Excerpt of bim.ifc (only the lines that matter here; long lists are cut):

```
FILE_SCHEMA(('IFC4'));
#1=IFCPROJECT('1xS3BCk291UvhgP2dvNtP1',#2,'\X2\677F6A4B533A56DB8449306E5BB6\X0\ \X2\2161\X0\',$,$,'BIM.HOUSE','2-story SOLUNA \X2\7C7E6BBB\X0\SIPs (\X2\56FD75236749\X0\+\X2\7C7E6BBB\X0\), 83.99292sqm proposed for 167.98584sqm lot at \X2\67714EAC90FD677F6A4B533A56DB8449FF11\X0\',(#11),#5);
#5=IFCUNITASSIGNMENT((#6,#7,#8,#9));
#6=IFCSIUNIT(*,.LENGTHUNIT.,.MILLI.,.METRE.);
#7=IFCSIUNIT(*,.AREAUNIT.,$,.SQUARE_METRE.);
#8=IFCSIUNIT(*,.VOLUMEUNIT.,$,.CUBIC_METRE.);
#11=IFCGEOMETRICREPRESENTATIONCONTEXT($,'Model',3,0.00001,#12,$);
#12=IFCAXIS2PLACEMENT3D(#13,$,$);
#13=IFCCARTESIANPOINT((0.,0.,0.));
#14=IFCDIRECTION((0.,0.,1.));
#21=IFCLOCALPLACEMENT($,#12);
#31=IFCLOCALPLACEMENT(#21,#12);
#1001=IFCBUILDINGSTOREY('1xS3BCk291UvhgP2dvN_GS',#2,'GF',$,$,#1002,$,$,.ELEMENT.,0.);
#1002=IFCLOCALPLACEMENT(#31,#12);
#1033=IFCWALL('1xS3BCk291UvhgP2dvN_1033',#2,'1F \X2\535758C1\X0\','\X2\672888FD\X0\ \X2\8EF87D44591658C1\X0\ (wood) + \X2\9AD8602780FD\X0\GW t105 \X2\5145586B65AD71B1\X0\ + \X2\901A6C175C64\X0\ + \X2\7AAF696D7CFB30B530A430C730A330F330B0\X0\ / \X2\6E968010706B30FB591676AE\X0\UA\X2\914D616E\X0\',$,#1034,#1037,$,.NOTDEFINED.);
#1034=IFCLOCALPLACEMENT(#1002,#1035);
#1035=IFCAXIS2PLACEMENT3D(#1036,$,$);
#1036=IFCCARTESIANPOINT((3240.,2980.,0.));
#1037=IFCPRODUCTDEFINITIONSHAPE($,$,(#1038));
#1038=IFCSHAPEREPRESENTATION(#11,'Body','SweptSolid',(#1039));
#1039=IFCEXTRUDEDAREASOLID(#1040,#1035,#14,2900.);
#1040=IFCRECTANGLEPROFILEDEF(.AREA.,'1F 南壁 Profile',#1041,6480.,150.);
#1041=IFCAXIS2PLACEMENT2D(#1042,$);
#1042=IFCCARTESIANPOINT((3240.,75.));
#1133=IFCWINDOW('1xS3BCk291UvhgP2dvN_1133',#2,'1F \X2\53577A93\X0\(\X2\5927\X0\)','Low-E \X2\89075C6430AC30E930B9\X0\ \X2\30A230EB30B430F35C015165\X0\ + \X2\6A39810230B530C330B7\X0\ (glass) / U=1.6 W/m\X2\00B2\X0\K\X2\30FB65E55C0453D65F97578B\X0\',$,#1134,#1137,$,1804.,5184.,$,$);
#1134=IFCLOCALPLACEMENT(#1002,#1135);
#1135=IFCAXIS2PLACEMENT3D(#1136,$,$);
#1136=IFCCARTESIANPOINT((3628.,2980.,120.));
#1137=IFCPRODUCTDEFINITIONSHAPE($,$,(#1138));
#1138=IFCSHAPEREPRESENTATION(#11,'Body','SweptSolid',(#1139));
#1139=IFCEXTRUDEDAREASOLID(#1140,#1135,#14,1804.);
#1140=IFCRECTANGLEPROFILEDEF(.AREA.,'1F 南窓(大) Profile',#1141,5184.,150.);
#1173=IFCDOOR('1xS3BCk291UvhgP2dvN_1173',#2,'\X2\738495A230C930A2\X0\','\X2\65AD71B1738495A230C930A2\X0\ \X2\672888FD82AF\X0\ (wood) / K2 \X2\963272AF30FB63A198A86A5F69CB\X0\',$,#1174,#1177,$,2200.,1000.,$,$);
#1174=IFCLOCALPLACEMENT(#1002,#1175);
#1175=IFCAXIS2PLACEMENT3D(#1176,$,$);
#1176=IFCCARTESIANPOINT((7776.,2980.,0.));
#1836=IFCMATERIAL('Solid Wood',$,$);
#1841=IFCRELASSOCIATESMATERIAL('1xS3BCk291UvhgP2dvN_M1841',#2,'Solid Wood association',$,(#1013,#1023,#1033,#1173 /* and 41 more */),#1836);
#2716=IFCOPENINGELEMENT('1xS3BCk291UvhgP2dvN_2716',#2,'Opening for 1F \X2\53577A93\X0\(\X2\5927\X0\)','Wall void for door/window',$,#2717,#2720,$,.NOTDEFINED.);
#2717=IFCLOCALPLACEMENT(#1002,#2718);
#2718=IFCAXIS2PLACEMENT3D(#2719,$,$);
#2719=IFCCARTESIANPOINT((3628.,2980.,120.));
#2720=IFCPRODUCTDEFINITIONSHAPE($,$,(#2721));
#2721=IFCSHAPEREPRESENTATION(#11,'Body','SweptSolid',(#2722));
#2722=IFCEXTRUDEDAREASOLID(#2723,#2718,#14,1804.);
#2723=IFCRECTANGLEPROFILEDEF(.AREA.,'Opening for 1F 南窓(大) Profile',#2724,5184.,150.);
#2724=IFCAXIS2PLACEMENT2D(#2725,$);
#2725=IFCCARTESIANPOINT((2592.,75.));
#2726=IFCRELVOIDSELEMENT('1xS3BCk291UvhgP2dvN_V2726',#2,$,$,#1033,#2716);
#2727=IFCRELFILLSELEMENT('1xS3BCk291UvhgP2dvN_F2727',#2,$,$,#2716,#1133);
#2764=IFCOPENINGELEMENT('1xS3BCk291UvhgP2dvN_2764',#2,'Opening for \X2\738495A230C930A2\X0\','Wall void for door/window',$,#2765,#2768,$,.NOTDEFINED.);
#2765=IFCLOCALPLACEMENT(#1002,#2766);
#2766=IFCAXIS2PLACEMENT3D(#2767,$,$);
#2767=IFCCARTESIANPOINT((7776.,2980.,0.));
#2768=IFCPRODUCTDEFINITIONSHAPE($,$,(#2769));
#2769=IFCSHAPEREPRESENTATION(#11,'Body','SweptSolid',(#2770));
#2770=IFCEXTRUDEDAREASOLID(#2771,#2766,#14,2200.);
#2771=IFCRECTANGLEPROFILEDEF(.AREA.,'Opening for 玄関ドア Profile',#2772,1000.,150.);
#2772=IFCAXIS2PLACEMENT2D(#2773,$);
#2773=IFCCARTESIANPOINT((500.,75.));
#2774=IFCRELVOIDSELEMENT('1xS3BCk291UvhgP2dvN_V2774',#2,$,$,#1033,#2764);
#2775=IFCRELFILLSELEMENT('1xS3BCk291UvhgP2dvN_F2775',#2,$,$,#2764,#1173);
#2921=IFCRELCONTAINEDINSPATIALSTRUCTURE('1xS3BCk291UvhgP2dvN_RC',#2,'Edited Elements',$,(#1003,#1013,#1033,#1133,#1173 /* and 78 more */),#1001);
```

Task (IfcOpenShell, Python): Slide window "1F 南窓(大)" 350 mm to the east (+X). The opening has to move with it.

```python
import ifcopenshell
import ifcopenshell.api.geometry
import ifcopenshell.util.placement
import ifcopenshell.util.unit

model = ifcopenshell.open("bim.ifc")
unit_scale = ifcopenshell.util.unit.calculate_unit_scale(model)

window = model.by_guid("1xS3BCk291UvhgP2dvN_1133")
opening = window.FillsVoids[0].RelatingOpeningElement
wall = opening.VoidsElements[0].RelatingBuildingElement

wall_matrix = ifcopenshell.util.placement.get_local_placement(wall.ObjectPlacement)
shift = wall_matrix[:3, 0] * 0.35 / unit_scale
before = ifcopenshell.util.placement.get_local_placement(window.ObjectPlacement)[:3, 3].copy()

# The window is not placed relative to its opening, so move both.
for product in (opening, window):
    matrix = ifcopenshell.util.placement.get_local_placement(product.ObjectPlacement)
    matrix[:3, 3] += shift
    ifcopenshell.api.geometry.edit_object_placement(model, product=product, matrix=matrix, is_si=False)

after = ifcopenshell.util.placement.get_local_placement(window.ObjectPlacement)[:3, 3]
print("window moved by", (after - before).round(3) + 0.0)

model.write("bim_rev.ifc")
```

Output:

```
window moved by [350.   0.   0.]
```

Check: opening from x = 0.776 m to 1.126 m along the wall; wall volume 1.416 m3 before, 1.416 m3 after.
